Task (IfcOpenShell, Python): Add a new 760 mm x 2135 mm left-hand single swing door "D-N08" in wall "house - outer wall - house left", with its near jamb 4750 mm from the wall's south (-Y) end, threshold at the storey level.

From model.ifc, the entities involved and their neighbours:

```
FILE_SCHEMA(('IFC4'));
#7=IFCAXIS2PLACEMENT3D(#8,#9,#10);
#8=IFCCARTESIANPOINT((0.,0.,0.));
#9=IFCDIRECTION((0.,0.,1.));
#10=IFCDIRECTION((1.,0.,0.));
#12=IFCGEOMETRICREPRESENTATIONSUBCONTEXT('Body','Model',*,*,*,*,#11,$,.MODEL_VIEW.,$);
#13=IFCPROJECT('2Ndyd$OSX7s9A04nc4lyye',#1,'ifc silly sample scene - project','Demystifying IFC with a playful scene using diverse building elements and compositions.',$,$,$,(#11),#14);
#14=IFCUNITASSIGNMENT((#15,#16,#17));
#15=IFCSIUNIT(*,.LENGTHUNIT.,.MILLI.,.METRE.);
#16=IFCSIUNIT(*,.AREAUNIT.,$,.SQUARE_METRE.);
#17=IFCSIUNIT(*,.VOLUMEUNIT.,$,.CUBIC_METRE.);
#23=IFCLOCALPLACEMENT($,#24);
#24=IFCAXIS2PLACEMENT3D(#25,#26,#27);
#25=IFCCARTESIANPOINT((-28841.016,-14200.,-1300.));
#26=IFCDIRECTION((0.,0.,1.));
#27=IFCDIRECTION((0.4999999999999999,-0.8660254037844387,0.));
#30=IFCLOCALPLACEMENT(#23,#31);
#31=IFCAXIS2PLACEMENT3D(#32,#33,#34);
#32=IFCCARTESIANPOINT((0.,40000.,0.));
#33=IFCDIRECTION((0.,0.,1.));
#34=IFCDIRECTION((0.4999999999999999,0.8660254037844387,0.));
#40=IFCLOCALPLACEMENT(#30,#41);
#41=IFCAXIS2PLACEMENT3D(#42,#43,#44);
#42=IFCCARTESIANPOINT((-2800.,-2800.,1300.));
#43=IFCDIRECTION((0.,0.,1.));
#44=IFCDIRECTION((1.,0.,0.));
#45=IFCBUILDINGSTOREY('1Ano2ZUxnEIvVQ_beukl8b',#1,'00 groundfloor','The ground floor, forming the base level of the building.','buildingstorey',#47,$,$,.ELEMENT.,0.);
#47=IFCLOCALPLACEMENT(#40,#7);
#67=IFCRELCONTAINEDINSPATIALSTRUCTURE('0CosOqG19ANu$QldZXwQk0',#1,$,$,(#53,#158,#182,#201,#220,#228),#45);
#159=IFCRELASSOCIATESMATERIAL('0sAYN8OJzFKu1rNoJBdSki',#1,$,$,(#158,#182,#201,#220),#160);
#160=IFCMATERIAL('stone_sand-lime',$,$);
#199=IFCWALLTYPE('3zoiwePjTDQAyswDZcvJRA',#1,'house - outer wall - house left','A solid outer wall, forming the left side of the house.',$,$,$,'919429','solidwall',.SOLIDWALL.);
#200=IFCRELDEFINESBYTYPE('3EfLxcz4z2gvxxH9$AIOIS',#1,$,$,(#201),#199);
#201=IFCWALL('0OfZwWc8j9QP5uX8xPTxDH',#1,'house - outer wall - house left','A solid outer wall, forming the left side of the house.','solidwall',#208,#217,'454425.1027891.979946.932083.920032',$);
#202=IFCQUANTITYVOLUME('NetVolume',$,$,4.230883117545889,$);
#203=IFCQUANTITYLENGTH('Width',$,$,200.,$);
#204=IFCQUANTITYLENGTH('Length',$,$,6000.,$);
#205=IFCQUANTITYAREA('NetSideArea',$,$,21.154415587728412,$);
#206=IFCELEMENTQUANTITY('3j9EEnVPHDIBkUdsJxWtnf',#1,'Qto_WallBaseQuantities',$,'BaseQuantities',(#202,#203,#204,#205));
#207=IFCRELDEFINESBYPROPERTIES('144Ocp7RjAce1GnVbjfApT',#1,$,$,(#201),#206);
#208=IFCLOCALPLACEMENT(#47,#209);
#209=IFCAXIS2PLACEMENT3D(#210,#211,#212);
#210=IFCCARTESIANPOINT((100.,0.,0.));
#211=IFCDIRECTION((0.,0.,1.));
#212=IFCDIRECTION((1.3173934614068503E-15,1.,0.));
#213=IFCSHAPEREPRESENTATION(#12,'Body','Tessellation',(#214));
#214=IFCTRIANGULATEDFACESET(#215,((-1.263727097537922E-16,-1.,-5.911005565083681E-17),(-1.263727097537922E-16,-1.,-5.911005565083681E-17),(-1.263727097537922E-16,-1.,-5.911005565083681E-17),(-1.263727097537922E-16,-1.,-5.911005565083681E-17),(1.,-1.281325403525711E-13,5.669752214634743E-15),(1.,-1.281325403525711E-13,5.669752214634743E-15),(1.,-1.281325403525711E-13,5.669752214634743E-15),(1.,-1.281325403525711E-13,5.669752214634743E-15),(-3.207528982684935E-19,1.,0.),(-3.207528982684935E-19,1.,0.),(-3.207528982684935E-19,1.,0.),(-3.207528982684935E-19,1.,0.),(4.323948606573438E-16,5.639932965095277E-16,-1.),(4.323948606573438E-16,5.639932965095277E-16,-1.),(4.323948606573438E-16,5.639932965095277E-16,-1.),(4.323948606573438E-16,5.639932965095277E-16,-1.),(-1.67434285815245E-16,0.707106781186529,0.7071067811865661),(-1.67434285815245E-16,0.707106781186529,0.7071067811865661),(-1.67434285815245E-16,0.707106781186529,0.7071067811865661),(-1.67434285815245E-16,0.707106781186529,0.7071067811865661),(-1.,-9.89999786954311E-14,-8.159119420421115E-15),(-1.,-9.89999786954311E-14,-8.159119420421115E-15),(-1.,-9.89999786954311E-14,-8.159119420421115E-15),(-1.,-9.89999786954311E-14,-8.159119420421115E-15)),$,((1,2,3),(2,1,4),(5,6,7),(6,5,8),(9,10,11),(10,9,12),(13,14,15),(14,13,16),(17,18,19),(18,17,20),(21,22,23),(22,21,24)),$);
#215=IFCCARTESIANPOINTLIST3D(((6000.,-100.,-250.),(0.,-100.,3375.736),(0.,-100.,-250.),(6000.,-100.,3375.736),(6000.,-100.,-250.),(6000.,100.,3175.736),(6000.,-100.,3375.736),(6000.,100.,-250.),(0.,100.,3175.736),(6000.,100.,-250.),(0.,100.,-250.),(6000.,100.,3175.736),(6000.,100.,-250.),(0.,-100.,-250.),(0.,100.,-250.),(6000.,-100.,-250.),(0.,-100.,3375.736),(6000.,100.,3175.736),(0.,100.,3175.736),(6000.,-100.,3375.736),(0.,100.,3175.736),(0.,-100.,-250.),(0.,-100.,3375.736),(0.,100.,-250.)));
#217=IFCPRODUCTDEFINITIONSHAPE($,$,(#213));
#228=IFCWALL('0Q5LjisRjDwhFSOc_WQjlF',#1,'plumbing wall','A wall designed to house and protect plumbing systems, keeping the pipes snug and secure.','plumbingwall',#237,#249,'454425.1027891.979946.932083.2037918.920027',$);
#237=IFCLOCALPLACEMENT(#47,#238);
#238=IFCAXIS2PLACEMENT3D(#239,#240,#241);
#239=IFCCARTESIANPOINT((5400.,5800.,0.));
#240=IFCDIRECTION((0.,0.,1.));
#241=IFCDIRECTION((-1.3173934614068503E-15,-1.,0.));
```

```python
import numpy as np
import ifcopenshell
import ifcopenshell.api.feature
import ifcopenshell.api.geometry
import ifcopenshell.api.pset
import ifcopenshell.api.root
import ifcopenshell.api.spatial
import ifcopenshell.geom
import ifcopenshell.util.element
import ifcopenshell.util.placement
import ifcopenshell.util.representation
import ifcopenshell.util.shape
import ifcopenshell.util.unit

model = ifcopenshell.open("model.ifc")
unit_scale = ifcopenshell.util.unit.calculate_unit_scale(model)
area_scale = ifcopenshell.util.unit.calculate_unit_scale(model, "AREAUNIT")
volume_scale = ifcopenshell.util.unit.calculate_unit_scale(model, "VOLUMEUNIT")
settings = ifcopenshell.geom.settings()


def volume(element):
    """Net volume in cubic metres, openings subtracted."""
    shape = ifcopenshell.geom.create_shape(settings, element)
    return ifcopenshell.util.shape.get_volume(shape.geometry)


wall = model.by_id(201)
storey = ifcopenshell.util.element.get_container(wall, ifc_class="IfcBuildingStorey")
context = ifcopenshell.util.representation.get_context(model, "Model", "Body", "MODEL_VIEW")
before = volume(wall)

width, height, from_end, sill = 0.76, 2.135, 4.75, 0.0  # metres

# The wall runs along its own X axis, and the end named is its -X end.
wall_shape = ifcopenshell.geom.create_shape(settings, wall)
x, y, z = ifcopenshell.util.shape.get_vertices(wall_shape.geometry).T
start = x.min() + from_end
face, thickness = float(y.min()), float(y.max() - y.min())
wall_matrix = ifcopenshell.util.placement.get_local_placement(wall.ObjectPlacement)
level = ifcopenshell.util.placement.get_local_placement(storey.ObjectPlacement)[2, 3]


def in_wall(x, y):
    """Placement at x, y metres in the wall's axes, at sill height."""
    matrix = wall_matrix.copy()
    matrix[:, 3] = wall_matrix @ np.array([x / unit_scale, y / unit_scale, 0.0, 1.0])
    matrix[2, 3] = level + sill / unit_scale
    return matrix


# Opening: a box that overshoots both wall faces by 50 mm.
opening = ifcopenshell.api.root.create_entity(model, ifc_class="IfcOpeningElement", predefined_type="OPENING")
box = ifcopenshell.api.geometry.add_wall_representation(
    model, context=context, length=width, height=height, thickness=thickness + 0.1
)
ifcopenshell.api.geometry.assign_representation(model, product=opening, representation=box)
ifcopenshell.api.geometry.edit_object_placement(model, product=opening, matrix=in_wall(start, face - 0.05), is_si=False)
ifcopenshell.api.feature.add_feature(model, feature=opening, element=wall)

door = ifcopenshell.api.root.create_entity(model, ifc_class="IfcDoor", name="D-N08", predefined_type="DOOR")
door.OverallWidth, door.OverallHeight = width / unit_scale, height / unit_scale
door.OperationType = "SINGLE_SWING_LEFT"
body = ifcopenshell.api.geometry.add_door_representation(
    model,
    context=context,
    overall_width=door.OverallWidth,
    overall_height=door.OverallHeight,
    operation_type="SINGLE_SWING_LEFT",
    lining_properties={"LiningDepth": thickness / unit_scale, "ThresholdDepth": thickness / unit_scale},
)
ifcopenshell.api.geometry.assign_representation(model, product=door, representation=body)
ifcopenshell.api.spatial.assign_container(model, products=[door], relating_structure=storey)
ifcopenshell.api.feature.add_filling(model, opening=opening, element=door)

# The lining spans the wall, so the door starts at the wall face.
ifcopenshell.api.geometry.edit_object_placement(model, product=door, matrix=in_wall(start, face), is_si=False)

after = volume(wall)

# Update the wall's stored quantities.
qto = model.by_id(ifcopenshell.util.element.get_pset(wall, "Qto_WallBaseQuantities", should_inherit=False)["id"])
ifcopenshell.api.pset.edit_qto(model, qto=qto, properties={
    "NetVolume": after / volume_scale,
    "NetSideArea": after / thickness / area_scale,
})

print(f"wall volume {before:.3f} -> {after:.3f} m3")

model.write("model_edited.ifc")
```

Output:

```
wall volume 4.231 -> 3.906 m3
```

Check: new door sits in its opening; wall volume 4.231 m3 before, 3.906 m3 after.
